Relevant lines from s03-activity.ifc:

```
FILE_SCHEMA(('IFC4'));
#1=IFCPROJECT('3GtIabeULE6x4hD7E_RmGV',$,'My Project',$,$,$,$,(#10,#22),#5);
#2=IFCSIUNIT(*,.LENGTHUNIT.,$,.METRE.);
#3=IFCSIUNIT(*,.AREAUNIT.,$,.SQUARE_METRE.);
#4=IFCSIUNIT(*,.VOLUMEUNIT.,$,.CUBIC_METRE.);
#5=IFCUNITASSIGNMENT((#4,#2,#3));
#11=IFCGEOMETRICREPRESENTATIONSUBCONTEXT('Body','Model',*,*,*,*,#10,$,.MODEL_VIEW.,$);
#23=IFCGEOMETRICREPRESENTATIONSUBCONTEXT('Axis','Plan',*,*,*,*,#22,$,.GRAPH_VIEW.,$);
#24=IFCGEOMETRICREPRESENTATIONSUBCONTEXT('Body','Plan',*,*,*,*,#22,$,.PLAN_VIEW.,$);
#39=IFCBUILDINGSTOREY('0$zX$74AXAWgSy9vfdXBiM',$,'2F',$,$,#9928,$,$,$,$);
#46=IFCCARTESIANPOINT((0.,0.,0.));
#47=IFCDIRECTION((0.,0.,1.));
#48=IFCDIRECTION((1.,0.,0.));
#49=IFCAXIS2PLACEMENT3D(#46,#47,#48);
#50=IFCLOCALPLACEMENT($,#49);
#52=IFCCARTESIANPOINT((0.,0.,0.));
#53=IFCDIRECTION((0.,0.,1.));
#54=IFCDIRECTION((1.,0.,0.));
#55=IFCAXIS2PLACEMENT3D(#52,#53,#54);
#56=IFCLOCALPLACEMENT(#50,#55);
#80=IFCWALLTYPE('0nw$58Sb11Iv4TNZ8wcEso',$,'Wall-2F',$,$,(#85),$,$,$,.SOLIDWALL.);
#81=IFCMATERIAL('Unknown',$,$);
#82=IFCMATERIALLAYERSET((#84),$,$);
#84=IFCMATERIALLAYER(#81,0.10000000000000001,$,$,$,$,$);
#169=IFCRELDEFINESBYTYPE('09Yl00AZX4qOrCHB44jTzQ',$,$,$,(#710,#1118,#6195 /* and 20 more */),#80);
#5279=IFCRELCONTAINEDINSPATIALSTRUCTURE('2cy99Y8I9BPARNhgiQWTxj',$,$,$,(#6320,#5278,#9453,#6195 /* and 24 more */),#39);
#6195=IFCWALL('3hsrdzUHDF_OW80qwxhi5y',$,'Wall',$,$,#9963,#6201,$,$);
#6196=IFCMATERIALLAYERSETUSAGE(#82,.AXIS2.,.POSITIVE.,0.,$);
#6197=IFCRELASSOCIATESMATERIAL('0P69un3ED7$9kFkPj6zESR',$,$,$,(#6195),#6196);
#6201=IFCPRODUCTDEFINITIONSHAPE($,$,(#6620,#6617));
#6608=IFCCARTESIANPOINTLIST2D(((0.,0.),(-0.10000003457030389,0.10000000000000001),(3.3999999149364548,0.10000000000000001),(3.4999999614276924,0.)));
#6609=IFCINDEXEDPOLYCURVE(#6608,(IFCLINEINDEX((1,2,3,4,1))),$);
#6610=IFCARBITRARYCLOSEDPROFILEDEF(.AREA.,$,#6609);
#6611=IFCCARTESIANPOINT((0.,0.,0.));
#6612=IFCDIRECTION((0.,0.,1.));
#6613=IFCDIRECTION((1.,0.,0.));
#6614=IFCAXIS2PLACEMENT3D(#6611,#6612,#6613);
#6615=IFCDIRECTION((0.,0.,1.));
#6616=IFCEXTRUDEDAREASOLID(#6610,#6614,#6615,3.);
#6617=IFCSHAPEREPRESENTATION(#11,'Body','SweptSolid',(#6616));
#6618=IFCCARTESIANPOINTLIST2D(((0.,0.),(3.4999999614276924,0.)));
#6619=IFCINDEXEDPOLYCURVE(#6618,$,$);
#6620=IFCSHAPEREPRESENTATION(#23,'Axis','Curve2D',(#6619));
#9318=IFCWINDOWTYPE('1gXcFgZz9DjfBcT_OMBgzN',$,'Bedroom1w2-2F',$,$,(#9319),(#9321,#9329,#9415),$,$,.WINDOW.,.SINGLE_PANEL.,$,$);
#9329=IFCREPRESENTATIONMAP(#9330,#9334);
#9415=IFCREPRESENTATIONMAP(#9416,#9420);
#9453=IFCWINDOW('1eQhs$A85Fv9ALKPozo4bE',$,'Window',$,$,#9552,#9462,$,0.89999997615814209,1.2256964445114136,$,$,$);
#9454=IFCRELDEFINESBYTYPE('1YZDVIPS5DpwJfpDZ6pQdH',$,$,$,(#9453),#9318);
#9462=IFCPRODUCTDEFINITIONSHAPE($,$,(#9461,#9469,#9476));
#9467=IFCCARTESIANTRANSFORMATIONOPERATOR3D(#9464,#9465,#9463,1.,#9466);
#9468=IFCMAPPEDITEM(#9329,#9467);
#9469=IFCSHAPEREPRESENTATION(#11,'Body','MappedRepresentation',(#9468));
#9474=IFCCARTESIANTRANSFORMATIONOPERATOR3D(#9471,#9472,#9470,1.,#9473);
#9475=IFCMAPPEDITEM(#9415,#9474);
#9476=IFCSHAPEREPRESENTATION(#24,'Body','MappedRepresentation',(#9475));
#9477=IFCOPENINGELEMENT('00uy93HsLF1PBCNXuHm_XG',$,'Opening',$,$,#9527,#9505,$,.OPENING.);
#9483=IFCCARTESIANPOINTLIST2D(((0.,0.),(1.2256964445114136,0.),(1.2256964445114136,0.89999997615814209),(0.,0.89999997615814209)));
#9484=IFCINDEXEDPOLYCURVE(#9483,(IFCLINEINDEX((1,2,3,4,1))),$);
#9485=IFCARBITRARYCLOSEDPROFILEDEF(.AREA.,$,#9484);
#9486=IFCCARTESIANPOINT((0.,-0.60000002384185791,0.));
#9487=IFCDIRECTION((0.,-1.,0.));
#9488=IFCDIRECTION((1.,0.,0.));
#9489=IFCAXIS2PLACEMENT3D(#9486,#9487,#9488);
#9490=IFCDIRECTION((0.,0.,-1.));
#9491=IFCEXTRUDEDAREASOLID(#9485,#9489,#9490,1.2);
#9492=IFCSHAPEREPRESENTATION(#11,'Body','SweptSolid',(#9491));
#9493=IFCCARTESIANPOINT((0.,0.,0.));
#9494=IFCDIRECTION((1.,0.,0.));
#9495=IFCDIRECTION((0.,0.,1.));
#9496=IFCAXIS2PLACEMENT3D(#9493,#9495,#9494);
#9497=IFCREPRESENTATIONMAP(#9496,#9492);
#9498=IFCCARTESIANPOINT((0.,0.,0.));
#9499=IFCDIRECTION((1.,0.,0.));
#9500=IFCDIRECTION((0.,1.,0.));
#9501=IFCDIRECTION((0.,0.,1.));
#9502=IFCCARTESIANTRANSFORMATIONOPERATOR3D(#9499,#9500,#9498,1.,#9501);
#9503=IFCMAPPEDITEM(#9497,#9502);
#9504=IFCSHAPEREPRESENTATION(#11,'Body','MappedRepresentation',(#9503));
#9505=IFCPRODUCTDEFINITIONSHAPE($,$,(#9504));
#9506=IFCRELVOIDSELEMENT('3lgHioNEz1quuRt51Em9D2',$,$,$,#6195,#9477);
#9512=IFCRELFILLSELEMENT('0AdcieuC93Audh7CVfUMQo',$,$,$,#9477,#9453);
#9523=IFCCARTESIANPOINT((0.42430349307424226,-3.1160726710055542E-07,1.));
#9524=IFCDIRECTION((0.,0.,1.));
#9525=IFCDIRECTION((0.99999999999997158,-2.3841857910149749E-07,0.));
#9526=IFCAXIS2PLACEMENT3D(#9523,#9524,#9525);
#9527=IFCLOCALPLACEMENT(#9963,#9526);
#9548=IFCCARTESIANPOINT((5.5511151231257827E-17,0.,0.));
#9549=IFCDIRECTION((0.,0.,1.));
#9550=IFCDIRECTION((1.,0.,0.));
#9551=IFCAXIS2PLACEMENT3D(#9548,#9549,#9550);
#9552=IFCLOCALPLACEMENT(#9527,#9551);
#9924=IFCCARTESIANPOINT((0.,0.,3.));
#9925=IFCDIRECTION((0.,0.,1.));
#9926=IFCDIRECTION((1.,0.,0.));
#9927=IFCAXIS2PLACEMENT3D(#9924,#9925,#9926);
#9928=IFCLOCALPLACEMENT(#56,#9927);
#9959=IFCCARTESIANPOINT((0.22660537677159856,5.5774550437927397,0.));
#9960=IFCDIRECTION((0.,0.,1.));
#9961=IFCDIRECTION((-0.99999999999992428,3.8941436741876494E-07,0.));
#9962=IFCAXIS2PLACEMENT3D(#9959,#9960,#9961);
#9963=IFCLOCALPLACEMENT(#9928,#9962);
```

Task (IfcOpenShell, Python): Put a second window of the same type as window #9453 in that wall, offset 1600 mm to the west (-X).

```python
import ifcopenshell
import ifcopenshell.api.feature
import ifcopenshell.api.geometry
import ifcopenshell.api.root
import ifcopenshell.geom
import ifcopenshell.util.element
import ifcopenshell.util.placement
import ifcopenshell.util.shape

model = ifcopenshell.open("s03-activity.ifc")
settings = ifcopenshell.geom.settings()


def volume(element):
    """Net volume in cubic metres, openings subtracted."""
    shape = ifcopenshell.geom.create_shape(settings, element)
    return ifcopenshell.util.shape.get_volume(shape.geometry)


window = model.by_id(9453)
opening = window.FillsVoids[0].RelatingOpeningElement
wall = opening.VoidsElements[0].RelatingBuildingElement
before = volume(wall)
shift = ifcopenshell.util.placement.get_local_placement(wall.ObjectPlacement)[:3, 0] * 1.6

# copy_class copies the void relationship, type, container and properties, but no geometry.
new_opening = ifcopenshell.api.root.copy_class(model, product=opening)
new_opening.Representation = ifcopenshell.util.element.copy_deep(
    model, opening.Representation, exclude=["IfcGeometricRepresentationContext", "IfcRepresentationMap"]
)
new_window = ifcopenshell.api.root.copy_class(model, product=window)
new_window.Representation = ifcopenshell.util.element.copy_deep(
    model, window.Representation, exclude=["IfcGeometricRepresentationContext", "IfcRepresentationMap"]
)
ifcopenshell.api.feature.add_filling(model, opening=new_opening, element=new_window)

for old, new in ((opening, new_opening), (window, new_window)):
    matrix = ifcopenshell.util.placement.get_local_placement(old.ObjectPlacement)
    matrix[:3, 3] += shift
    ifcopenshell.api.geometry.edit_object_placement(model, product=new, matrix=matrix, is_si=False)

after = volume(wall)

print(f"wall volume {before:.3f} -> {after:.3f} m3")

model.write("s03-activity_rev.ifc")
```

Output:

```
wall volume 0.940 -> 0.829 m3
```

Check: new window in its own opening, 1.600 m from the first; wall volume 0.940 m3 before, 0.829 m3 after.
